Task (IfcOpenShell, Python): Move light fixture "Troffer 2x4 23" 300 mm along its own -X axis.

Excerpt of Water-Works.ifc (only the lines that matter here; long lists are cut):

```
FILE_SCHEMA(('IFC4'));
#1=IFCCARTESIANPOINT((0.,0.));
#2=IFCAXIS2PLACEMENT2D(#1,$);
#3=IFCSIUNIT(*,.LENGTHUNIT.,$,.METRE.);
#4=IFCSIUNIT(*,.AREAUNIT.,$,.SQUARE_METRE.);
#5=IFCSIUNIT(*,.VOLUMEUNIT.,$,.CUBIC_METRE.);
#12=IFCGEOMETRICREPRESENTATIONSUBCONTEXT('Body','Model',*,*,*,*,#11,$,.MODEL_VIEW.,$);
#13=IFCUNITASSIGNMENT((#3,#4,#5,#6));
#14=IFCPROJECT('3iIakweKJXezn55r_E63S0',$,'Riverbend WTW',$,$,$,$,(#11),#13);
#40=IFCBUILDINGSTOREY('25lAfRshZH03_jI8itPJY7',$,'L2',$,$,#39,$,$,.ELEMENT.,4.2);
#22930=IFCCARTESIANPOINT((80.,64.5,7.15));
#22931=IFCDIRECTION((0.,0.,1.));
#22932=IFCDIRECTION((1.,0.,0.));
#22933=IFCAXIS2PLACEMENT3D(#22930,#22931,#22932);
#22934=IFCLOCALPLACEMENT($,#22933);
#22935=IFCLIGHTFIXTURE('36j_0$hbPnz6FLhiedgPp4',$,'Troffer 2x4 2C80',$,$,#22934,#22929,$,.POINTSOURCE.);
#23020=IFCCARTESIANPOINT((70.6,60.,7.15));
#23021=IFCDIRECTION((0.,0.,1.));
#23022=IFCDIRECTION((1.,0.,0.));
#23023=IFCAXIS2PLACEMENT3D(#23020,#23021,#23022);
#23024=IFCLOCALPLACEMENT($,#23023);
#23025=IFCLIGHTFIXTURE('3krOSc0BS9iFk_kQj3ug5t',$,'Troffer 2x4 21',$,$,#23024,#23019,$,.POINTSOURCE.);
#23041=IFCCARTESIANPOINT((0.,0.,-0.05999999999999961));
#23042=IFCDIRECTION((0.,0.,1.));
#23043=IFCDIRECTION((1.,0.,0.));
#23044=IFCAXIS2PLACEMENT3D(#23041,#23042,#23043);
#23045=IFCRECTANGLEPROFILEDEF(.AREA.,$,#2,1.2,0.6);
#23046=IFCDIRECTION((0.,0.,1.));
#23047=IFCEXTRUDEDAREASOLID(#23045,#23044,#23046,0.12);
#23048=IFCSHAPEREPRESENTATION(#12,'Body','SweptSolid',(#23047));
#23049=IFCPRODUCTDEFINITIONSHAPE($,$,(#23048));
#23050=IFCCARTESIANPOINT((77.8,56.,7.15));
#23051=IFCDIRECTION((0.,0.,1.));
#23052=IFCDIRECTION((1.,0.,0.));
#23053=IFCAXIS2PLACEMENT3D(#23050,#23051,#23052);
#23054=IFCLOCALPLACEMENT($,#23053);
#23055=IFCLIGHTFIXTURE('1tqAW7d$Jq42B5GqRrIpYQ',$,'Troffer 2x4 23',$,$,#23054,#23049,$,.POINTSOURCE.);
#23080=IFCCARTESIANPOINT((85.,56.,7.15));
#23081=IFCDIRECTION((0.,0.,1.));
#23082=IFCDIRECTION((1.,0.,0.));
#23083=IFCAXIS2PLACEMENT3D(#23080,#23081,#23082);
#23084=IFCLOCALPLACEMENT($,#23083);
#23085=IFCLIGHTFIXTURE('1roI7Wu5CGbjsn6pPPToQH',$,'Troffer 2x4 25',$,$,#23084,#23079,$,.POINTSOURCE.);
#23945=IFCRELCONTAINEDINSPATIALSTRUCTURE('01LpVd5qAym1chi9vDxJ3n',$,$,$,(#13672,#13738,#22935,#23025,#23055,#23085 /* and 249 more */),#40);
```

```python
import ifcopenshell
import ifcopenshell.api.geometry
import ifcopenshell.util.placement
import ifcopenshell.util.unit

model = ifcopenshell.open("Water-Works.ifc")
unit_scale = ifcopenshell.util.unit.calculate_unit_scale(model)

item = model.by_id(23055)
matrix = ifcopenshell.util.placement.get_local_placement(item.ObjectPlacement)
matrix[:3, 3] -= matrix[:3, 0] * 0.3 / unit_scale
ifcopenshell.api.geometry.edit_object_placement(model, product=item, matrix=matrix, is_si=False)

print(ifcopenshell.util.placement.get_local_placement(item.ObjectPlacement).round(3) + 0.0)

model.write("Water-Works_updated.ifc")
```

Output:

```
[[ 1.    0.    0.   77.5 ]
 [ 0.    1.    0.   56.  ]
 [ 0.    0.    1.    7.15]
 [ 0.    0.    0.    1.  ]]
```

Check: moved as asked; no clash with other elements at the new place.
